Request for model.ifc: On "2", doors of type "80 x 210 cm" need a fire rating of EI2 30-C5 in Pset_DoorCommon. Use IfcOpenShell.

First a look at what the model holds.

```python
import ifcopenshell
import ifcopenshell.util.element

model = ifcopenshell.open("model.ifc")
print(model.schema)
storey = next(s for s in model.by_type("IfcBuildingStorey") if s.Name == "2")
doors = [e for e in ifcopenshell.util.element.get_decomposition(storey) if e.is_a("IfcDoor")]
seen = {}
for e in doors:
    element_type = ifcopenshell.util.element.get_type(e)
    key = (element_type.Name if element_type != e and element_type else None, ifcopenshell.util.element.get_pset(e, "Pset_DoorCommon", "FireRating"))
    seen[key] = seen.get(key, 0) + 1
for (name, value), count in sorted(seen.items(), key=str):
    print(count, "x", name, "|", value)
```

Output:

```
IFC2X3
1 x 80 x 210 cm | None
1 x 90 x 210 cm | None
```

```python
import ifcopenshell
import ifcopenshell.api.pset
import ifcopenshell.util.element

model = ifcopenshell.open("model.ifc")

storey = next(s for s in model.by_type("IfcBuildingStorey") if s.Name == "2")
doors = [e for e in ifcopenshell.util.element.get_decomposition(storey) if e.is_a("IfcDoor")]

count = 0
for e in doors:
    element_type = ifcopenshell.util.element.get_type(e)
    if element_type in (None, e) or element_type.Name != "80 x 210 cm":
        continue
    # add_pset returns the element's existing set when there is one.
    pset = ifcopenshell.api.pset.add_pset(model, product=e, name="Pset_DoorCommon")
    ifcopenshell.api.pset.edit_pset(model, pset=pset, properties={"FireRating": "EI2 30-C5"})
    count += 1

print(count, "doors updated")

model.write("model_updated.ifc")
```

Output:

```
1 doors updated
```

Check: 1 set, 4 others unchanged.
